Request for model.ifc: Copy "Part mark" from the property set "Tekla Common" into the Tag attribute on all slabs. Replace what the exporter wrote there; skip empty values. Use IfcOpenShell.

First a look at what the model holds.

```python
import ifcopenshell
import ifcopenshell.util.element

model = ifcopenshell.open("model.ifc")
print(model.schema)
slabs = model.by_type("IfcSlab")
print(len(slabs), "slabs")
for e in slabs[:8]:
    source = ifcopenshell.util.element.get_pset(e, "Tekla Common", "Part mark")
    target = e.Tag
    print(e.id(), repr(source), repr(target), sep=" | ")
```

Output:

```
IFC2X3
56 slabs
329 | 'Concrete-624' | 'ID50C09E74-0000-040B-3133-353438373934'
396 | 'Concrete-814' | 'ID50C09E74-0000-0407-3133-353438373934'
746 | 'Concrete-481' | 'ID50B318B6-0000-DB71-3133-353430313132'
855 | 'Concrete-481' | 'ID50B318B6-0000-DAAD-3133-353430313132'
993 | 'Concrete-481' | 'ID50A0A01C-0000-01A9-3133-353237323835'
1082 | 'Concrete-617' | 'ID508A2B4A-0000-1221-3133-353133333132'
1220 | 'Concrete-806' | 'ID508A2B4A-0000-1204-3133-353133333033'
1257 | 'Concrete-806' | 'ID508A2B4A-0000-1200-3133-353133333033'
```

```python
import ifcopenshell
import ifcopenshell.util.element

model = ifcopenshell.open("model.ifc")

count = 0
for e in model.by_type("IfcSlab"):
    value = ifcopenshell.util.element.get_pset(e, "Tekla Common", "Part mark")
    current = e.Tag
    if not value or not value.strip() or current == value:
        continue
    e.Tag = value
    count += 1

print(count, "slabs updated")

model.write("model_updated.ifc")
```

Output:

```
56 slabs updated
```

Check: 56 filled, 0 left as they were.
